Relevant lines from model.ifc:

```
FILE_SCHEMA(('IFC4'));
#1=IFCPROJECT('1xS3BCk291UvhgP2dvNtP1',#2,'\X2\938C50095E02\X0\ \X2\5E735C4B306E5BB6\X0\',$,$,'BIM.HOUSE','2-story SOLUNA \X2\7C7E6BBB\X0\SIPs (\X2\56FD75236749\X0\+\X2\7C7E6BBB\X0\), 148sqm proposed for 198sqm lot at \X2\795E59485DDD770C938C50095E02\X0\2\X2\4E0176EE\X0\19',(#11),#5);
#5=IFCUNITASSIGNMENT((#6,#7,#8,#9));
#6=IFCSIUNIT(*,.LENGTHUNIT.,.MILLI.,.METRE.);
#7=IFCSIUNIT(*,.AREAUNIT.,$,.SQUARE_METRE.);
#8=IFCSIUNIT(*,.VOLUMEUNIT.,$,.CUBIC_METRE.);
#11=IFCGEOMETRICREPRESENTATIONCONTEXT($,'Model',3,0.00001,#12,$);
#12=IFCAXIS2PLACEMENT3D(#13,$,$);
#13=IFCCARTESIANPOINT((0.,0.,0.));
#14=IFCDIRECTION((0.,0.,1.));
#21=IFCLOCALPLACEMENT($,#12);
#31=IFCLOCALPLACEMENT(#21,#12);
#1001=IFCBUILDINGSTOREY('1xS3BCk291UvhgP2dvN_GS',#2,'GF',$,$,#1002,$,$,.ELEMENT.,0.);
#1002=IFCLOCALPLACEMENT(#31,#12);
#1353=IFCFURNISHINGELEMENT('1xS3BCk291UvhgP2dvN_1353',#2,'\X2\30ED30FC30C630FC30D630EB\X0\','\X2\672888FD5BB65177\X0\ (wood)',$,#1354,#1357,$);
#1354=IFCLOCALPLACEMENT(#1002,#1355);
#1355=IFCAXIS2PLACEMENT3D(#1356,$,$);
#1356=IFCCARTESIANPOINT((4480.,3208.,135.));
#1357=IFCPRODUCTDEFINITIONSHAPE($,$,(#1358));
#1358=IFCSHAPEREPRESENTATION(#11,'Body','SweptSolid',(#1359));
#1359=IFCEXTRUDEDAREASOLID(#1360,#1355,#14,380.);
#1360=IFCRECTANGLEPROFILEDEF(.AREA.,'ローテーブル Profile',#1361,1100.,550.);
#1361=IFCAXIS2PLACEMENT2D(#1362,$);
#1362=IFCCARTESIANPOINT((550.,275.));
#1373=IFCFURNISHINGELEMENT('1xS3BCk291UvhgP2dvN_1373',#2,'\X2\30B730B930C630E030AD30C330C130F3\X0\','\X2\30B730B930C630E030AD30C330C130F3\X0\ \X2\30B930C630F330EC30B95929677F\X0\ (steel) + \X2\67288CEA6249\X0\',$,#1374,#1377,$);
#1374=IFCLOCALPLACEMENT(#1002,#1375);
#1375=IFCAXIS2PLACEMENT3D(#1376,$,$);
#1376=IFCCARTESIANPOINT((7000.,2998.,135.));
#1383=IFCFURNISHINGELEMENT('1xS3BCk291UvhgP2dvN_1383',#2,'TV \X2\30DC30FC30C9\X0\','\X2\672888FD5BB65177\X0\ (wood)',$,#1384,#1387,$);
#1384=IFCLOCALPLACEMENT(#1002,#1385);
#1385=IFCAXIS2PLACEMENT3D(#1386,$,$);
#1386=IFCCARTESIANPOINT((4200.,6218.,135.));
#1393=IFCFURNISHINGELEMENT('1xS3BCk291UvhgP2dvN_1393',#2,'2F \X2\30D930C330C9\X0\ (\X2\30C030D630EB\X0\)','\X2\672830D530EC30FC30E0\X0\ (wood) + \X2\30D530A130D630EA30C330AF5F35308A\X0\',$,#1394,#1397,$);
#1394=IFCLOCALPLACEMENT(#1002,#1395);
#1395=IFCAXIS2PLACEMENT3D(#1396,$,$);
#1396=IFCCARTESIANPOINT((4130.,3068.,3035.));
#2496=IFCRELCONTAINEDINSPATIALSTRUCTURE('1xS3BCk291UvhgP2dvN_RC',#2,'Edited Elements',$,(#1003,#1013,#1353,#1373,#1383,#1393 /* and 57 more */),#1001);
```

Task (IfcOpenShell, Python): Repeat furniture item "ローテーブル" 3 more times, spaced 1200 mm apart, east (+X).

```python
import numpy as np
import ifcopenshell
import ifcopenshell.api.geometry
import ifcopenshell.api.root
import ifcopenshell.util.element
import ifcopenshell.util.placement

model = ifcopenshell.open("model.ifc")


def reuse_history(source, copy):
    """copy_class also copies each property set's owner history, people and application; keep the originals."""
    for rel in copy.IsDefinedBy:
        if rel.is_a("IfcRelDefinesByProperties") and (history := rel.RelatingPropertyDefinition.OwnerHistory):
            rel.RelatingPropertyDefinition.OwnerHistory = source.OwnerHistory
            ifcopenshell.util.element.remove_deep2(model, history)


source = model.by_id(1353)
base = ifcopenshell.util.placement.get_local_placement(source.ObjectPlacement)
step = np.array([1.0, 0.0, 0.0]) * 1200.0

for i in range(1, 4):
    copy = ifcopenshell.api.root.copy_class(model, product=source)
    copy.Representation = ifcopenshell.util.element.copy_deep(
        model, source.Representation, exclude=["IfcGeometricRepresentationContext", "IfcRepresentationMap"]
    )
    reuse_history(source, copy)
    matrix = base.copy()
    matrix[:3, 3] += i * step
    print("added at", matrix[:3, 3].round(3) + 0.0)
    ifcopenshell.api.geometry.edit_object_placement(model, product=copy, matrix=matrix, is_si=False)

model.write("model_rev.ifc")
```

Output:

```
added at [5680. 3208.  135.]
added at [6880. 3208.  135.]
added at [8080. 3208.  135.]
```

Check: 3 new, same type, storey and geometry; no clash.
